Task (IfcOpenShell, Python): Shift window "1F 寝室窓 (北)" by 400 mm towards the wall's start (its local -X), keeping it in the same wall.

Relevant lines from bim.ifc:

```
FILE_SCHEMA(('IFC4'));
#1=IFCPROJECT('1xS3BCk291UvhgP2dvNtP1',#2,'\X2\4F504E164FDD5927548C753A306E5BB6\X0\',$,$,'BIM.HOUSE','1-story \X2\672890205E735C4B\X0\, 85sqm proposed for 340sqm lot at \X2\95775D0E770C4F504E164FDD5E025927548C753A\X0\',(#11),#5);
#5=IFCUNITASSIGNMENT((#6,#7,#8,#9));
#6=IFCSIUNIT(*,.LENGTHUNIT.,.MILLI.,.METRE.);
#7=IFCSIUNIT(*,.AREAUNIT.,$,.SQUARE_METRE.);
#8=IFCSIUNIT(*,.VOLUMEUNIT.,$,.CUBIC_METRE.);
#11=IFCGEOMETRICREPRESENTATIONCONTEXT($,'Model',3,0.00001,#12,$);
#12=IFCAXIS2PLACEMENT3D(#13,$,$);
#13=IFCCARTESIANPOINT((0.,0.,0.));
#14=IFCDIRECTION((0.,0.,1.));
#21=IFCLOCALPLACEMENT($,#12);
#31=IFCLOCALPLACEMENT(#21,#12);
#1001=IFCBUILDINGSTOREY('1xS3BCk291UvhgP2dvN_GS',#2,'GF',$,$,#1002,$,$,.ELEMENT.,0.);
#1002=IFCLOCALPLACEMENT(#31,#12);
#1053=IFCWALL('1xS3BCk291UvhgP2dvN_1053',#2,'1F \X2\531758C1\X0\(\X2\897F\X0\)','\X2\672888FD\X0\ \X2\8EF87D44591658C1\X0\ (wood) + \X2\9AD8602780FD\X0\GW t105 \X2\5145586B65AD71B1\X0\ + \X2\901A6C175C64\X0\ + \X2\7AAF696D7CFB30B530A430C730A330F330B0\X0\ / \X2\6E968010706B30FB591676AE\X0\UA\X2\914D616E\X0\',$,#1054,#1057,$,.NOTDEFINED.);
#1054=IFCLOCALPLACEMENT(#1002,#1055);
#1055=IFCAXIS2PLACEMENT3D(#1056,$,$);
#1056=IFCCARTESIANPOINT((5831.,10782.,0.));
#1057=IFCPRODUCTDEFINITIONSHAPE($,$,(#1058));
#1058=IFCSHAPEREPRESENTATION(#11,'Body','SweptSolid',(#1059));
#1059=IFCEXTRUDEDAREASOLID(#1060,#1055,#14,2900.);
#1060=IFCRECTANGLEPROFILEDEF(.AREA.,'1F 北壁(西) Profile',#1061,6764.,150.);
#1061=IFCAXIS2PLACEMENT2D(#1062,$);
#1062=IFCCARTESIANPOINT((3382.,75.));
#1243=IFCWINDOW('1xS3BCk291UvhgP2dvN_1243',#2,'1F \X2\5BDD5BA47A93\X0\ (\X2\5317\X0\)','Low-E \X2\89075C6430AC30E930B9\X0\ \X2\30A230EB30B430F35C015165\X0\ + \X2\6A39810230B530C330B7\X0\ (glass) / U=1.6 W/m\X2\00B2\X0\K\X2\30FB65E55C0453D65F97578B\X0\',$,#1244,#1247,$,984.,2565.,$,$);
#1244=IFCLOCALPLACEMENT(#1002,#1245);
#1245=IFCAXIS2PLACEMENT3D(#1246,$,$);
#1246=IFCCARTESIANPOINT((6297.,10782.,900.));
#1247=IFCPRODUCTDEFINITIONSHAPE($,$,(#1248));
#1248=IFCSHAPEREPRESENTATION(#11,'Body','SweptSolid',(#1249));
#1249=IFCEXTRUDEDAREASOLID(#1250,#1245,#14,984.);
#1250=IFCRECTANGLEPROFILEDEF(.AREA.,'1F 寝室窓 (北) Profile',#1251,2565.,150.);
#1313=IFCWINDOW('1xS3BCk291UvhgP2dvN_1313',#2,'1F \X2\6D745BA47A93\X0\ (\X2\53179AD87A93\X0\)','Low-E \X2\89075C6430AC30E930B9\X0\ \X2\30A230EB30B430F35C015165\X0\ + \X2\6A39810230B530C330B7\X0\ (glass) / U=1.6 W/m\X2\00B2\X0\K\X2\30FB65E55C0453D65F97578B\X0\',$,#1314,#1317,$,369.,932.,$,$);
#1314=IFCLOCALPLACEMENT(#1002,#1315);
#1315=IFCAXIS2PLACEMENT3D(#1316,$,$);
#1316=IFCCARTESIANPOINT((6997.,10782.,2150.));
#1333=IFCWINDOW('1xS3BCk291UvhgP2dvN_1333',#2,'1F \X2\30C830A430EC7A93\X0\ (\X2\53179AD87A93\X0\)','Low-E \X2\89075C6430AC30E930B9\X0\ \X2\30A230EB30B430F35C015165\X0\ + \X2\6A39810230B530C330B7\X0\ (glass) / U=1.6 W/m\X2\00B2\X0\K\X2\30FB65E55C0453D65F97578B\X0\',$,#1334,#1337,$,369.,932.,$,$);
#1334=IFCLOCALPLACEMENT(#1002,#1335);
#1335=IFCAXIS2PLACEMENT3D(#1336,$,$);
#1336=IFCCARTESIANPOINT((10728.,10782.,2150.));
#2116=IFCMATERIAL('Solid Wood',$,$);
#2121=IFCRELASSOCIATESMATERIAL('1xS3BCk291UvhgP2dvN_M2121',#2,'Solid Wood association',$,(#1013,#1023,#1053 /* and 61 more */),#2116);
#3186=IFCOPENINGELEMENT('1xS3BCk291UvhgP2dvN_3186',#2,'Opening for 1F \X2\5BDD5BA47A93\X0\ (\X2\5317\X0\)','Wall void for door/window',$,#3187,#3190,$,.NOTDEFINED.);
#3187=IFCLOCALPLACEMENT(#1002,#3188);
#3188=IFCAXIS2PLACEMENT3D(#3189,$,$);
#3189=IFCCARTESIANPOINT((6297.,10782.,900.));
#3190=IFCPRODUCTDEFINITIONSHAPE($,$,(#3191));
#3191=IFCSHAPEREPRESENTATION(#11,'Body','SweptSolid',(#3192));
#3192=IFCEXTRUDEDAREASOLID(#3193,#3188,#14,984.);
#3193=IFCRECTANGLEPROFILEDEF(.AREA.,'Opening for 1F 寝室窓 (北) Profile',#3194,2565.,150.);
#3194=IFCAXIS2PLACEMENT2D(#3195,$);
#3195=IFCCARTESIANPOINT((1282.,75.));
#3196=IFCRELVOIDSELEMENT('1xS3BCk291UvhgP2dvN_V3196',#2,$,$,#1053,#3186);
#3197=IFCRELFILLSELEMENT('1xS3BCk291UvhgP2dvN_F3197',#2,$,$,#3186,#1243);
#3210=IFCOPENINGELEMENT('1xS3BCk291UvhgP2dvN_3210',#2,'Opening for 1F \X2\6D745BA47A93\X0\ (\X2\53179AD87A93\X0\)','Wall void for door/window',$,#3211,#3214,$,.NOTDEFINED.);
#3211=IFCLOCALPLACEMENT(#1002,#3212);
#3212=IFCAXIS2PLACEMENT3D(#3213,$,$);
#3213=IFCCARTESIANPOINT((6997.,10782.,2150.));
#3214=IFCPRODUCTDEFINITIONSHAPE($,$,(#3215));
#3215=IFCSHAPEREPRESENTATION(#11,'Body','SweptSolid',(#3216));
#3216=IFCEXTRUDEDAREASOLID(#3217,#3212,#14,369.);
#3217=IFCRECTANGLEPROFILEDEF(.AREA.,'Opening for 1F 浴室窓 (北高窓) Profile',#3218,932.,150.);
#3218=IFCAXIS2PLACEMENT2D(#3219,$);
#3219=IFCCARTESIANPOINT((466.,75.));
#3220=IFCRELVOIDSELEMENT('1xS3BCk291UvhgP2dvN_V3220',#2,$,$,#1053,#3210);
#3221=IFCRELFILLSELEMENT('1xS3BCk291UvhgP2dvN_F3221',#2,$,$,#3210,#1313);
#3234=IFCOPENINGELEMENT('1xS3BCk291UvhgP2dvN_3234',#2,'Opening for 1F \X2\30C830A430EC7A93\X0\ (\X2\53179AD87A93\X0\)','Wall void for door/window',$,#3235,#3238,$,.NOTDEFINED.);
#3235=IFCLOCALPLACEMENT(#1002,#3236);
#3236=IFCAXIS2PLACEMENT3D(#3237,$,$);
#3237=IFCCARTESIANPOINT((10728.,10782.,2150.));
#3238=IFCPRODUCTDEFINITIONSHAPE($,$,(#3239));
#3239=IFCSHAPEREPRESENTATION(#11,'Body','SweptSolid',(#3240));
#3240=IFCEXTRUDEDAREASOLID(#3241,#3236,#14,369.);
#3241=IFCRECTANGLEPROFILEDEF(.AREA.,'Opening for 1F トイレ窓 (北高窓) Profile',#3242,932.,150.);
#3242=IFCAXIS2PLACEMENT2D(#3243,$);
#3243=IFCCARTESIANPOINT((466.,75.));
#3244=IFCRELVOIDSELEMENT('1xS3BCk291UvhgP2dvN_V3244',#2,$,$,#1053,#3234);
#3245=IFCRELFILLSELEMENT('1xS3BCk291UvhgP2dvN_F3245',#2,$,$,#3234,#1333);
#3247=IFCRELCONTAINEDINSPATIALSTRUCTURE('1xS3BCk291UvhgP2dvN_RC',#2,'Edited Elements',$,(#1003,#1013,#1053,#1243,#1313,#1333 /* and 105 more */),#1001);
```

```python
import ifcopenshell
import ifcopenshell.api.geometry
import ifcopenshell.util.placement
import ifcopenshell.util.unit

model = ifcopenshell.open("bim.ifc")
unit_scale = ifcopenshell.util.unit.calculate_unit_scale(model)

window = model.by_guid("1xS3BCk291UvhgP2dvN_1243")
opening = window.FillsVoids[0].RelatingOpeningElement
wall = opening.VoidsElements[0].RelatingBuildingElement

wall_matrix = ifcopenshell.util.placement.get_local_placement(wall.ObjectPlacement)
shift = wall_matrix[:3, 0] * -0.4 / unit_scale
before = ifcopenshell.util.placement.get_local_placement(window.ObjectPlacement)[:3, 3].copy()

# The window is not placed relative to its opening, so move both.
for product in (opening, window):
    matrix = ifcopenshell.util.placement.get_local_placement(product.ObjectPlacement)
    matrix[:3, 3] += shift
    ifcopenshell.api.geometry.edit_object_placement(model, product=product, matrix=matrix, is_si=False)

after = ifcopenshell.util.placement.get_local_placement(window.ObjectPlacement)[:3, 3]
print("window moved by", (after - before).round(3) + 0.0)

model.write("bim_edited.ifc")
```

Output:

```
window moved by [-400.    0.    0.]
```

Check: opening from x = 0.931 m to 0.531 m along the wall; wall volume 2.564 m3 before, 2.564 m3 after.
